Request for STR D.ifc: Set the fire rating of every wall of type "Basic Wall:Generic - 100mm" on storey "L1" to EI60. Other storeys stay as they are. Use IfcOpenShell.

First a look at what the model holds.

```python
import ifcopenshell
import ifcopenshell.util.element

model = ifcopenshell.open("STR D.ifc")
print(model.schema)
storey = next(s for s in model.by_type("IfcBuildingStorey") if s.Name == "L1")
walls = [e for e in ifcopenshell.util.element.get_decomposition(storey) if e.is_a("IfcWall")]
seen = {}
for e in walls:
    element_type = ifcopenshell.util.element.get_type(e)
    key = (element_type.Name if element_type != e and element_type else None, ifcopenshell.util.element.get_pset(e, "Pset_WallCommon", "FireRating"))
    seen[key] = seen.get(key, 0) + 1
for (name, value), count in sorted(seen.items(), key=str):
    print(count, "x", name, "|", value)
```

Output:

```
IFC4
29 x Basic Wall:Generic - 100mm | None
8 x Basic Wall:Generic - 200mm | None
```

```python
import ifcopenshell
import ifcopenshell.api.pset
import ifcopenshell.util.element

model = ifcopenshell.open("STR D.ifc")

storey = next(s for s in model.by_type("IfcBuildingStorey") if s.Name == "L1")
walls = [e for e in ifcopenshell.util.element.get_decomposition(storey) if e.is_a("IfcWall")]

count = 0
for e in walls:
    element_type = ifcopenshell.util.element.get_type(e)
    if element_type in (None, e) or element_type.Name != "Basic Wall:Generic - 100mm":
        continue
    # add_pset returns the element's existing set when there is one.
    pset = ifcopenshell.api.pset.add_pset(model, product=e, name="Pset_WallCommon")
    ifcopenshell.api.pset.edit_pset(model, pset=pset, properties={"FireRating": "EI60"})
    count += 1

print(count, "walls updated")

model.write("STR D_rev.ifc")
```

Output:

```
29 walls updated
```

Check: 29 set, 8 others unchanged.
